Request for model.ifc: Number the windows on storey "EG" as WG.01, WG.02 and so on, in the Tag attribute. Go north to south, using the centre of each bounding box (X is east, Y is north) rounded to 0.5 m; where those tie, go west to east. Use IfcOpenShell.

First a look at what the model holds.

```python
import ifcopenshell
import ifcopenshell.util.element
import ifcopenshell.util.placement

model = ifcopenshell.open("model.ifc")
print(model.schema)
storey = next(s for s in model.by_type("IfcBuildingStorey") if s.Name == "EG")
windows = [e for e in ifcopenshell.util.element.get_decomposition(storey) if e.is_a("IfcWindow")]
for e in sorted(windows, key=lambda e: e.id()):
    origin = ifcopenshell.util.placement.get_local_placement(e.ObjectPlacement)[:3, 3]
    print(e.id(), e.Tag, e.Name, origin.round(2) + 0.0, sep=" | ")
```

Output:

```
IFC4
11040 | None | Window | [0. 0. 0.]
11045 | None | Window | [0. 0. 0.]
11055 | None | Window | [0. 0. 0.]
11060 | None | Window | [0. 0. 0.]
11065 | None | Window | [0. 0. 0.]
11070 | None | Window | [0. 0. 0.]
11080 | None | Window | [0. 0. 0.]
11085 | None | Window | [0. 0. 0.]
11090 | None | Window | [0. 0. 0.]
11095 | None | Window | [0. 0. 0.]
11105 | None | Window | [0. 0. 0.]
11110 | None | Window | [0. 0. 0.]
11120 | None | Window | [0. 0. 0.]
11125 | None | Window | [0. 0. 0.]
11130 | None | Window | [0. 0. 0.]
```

```python
import ifcopenshell
import ifcopenshell.geom
import ifcopenshell.util.element
import ifcopenshell.util.shape

model = ifcopenshell.open("model.ifc")
settings = ifcopenshell.geom.settings()
settings.set("use-world-coords", True)


def centre(element):
    shape = ifcopenshell.geom.create_shape(settings, element)
    return ifcopenshell.util.shape.get_bbox_centroid(shape.geometry)


storey = next(s for s in model.by_type("IfcBuildingStorey") if s.Name == "EG")
windows = [e for e in ifcopenshell.util.element.get_decomposition(storey) if e.is_a("IfcWindow")]

# Insertion points can sit at a corner or the storey origin, so sort by the geometry (in metres).
centres = {e: centre(e) for e in windows}
windows.sort(key=lambda e: (-round(centres[e][1] / 0.5), centres[e][0]))

for i, e in enumerate(windows, start=1):
    number = f"WG.{i:02d}"
    e.Tag = number
    print(e.id(), number)

model.write("model_edited.ifc")
```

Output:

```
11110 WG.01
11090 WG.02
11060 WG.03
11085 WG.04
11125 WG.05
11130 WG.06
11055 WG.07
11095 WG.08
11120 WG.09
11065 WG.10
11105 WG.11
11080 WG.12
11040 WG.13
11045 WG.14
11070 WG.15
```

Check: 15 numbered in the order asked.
